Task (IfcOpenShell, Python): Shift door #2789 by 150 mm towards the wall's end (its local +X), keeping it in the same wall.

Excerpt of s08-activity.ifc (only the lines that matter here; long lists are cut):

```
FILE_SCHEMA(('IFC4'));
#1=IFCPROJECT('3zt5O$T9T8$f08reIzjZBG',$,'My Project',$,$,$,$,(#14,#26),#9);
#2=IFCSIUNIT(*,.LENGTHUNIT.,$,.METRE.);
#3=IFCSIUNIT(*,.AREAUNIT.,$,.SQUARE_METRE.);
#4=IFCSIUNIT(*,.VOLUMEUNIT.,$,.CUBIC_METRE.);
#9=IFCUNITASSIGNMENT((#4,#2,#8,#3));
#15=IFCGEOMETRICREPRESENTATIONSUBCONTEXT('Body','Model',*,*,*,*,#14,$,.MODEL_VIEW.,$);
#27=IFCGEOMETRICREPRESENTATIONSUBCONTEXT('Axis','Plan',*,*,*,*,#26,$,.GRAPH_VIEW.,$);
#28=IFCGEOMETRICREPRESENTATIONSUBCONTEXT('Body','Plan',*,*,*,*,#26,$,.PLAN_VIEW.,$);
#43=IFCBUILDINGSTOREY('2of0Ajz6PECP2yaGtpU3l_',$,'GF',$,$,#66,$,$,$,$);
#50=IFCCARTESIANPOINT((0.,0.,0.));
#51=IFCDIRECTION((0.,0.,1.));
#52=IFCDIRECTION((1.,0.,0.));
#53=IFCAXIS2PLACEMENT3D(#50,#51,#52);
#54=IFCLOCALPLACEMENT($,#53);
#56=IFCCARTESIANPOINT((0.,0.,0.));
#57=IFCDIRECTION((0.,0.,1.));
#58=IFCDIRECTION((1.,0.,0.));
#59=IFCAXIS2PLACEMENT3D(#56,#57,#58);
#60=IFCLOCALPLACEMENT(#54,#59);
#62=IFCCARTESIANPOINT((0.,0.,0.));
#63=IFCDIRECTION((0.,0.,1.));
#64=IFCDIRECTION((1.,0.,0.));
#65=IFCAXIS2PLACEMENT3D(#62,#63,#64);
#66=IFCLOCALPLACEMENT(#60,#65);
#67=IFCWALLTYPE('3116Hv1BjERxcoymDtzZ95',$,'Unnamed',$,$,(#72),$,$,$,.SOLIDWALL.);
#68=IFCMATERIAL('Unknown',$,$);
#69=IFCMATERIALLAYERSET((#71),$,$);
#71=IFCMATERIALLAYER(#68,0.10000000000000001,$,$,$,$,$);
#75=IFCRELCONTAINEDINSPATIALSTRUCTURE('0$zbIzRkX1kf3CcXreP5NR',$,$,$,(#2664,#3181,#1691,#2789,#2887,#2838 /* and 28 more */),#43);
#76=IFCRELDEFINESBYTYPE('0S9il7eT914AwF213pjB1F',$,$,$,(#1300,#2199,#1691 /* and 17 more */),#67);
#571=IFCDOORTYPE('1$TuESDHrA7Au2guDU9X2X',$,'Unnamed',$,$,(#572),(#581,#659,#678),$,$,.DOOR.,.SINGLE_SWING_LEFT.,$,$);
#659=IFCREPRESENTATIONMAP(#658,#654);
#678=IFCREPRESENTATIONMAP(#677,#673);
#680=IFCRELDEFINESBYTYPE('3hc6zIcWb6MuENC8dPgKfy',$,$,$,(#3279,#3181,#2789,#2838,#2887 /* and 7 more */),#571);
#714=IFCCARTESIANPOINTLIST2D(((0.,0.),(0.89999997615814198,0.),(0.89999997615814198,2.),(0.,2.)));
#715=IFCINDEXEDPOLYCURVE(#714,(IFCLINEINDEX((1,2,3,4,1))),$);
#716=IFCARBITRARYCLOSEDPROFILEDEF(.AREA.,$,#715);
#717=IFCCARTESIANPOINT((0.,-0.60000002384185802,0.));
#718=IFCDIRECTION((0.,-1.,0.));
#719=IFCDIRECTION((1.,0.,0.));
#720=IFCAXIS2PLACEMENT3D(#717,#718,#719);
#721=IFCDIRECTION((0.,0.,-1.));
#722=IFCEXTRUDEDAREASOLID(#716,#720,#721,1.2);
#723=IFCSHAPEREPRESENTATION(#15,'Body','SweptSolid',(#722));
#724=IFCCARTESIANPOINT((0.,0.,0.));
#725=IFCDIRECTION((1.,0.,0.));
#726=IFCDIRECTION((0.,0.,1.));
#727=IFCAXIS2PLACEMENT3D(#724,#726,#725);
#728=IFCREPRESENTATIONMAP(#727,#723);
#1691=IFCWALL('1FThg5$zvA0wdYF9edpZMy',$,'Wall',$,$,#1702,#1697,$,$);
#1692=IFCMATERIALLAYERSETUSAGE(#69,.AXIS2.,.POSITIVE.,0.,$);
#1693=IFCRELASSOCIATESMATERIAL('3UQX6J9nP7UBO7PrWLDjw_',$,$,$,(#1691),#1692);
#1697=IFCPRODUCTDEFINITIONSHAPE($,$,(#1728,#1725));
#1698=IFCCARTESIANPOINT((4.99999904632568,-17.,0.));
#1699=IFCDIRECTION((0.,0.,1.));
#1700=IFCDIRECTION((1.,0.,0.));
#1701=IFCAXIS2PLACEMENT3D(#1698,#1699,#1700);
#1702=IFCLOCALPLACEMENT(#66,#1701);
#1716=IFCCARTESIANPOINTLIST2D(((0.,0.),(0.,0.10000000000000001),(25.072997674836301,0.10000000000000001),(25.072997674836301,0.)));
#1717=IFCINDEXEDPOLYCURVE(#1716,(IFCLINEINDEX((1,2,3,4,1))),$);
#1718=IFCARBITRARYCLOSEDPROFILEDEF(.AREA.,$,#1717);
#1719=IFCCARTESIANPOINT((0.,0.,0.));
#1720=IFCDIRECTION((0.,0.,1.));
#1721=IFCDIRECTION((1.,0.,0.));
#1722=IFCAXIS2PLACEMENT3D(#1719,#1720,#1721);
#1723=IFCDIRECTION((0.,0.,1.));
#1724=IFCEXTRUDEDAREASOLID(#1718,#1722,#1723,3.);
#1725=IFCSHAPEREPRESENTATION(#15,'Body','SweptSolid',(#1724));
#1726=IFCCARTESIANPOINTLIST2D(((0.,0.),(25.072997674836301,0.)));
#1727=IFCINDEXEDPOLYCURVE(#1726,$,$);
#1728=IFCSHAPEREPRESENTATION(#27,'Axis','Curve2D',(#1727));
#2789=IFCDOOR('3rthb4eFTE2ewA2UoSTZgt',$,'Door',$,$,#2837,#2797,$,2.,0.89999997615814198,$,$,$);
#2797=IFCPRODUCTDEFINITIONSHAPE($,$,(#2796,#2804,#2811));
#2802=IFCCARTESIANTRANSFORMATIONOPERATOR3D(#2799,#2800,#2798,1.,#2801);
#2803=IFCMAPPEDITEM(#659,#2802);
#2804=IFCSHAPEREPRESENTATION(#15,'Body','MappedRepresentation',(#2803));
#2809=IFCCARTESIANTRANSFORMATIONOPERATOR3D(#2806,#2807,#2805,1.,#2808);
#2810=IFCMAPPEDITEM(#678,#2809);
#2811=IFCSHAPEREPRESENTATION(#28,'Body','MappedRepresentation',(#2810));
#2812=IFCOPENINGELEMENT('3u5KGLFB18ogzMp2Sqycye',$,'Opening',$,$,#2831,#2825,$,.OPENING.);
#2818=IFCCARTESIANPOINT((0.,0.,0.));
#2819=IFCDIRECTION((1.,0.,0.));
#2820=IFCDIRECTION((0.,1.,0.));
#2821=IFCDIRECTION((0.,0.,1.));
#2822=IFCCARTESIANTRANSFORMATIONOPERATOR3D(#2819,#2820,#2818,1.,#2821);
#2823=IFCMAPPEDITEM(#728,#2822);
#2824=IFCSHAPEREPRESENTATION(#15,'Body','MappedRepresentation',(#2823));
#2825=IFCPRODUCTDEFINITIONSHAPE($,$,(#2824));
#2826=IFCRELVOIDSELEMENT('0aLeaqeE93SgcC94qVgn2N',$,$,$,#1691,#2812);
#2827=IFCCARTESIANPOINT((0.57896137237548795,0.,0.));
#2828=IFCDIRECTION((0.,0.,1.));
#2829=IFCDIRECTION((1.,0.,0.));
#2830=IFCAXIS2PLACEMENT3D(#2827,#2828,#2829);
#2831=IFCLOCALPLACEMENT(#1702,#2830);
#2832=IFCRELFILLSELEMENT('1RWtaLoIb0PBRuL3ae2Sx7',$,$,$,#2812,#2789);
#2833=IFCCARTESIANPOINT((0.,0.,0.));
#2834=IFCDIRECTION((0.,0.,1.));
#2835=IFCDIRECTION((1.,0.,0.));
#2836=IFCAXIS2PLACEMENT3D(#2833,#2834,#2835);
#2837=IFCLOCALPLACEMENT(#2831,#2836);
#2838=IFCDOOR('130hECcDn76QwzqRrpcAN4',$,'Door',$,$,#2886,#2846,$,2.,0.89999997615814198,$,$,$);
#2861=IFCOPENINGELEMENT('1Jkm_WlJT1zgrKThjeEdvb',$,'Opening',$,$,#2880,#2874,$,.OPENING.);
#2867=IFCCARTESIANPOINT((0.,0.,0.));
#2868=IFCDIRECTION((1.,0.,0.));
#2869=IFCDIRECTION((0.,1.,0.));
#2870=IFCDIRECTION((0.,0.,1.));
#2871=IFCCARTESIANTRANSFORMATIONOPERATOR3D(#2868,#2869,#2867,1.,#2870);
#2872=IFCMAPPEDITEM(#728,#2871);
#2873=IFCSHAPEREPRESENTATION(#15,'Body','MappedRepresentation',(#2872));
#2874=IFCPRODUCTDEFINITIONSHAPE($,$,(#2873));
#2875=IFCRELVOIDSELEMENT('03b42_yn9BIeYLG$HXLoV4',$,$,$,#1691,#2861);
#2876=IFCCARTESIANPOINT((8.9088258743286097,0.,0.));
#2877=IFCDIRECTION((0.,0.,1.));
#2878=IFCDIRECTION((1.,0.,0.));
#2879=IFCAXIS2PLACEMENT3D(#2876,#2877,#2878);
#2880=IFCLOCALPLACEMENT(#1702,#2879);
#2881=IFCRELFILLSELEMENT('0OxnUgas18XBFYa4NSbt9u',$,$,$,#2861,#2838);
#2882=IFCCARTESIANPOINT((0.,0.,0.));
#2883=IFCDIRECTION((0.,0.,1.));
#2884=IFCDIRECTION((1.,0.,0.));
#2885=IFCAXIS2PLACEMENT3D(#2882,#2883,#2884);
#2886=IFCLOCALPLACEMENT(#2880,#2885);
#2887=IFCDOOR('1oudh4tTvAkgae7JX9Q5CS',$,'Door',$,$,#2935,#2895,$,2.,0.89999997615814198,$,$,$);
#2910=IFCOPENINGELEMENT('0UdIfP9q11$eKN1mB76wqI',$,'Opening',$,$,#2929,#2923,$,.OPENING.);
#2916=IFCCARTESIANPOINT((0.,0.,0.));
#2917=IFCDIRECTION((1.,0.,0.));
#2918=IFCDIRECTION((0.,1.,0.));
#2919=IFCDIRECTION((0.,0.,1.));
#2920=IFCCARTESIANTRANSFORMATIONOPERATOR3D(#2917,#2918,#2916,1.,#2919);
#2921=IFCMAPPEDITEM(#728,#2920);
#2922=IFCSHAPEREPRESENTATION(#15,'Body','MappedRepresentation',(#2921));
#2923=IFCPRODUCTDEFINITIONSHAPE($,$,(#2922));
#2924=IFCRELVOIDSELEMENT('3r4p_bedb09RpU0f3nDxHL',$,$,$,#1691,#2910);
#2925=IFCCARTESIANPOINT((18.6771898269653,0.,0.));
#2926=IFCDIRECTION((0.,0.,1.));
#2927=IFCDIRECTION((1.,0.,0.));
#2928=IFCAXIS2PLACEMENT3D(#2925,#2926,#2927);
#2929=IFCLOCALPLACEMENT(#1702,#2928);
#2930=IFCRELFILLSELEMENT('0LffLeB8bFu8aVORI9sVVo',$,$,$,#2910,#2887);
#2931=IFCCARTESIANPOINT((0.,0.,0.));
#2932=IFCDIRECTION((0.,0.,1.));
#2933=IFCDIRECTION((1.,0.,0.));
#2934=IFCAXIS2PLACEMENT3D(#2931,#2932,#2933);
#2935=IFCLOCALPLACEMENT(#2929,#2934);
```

```python
import ifcopenshell
import ifcopenshell.api.geometry
import ifcopenshell.util.placement

model = ifcopenshell.open("s08-activity.ifc")

door = model.by_guid("3rthb4eFTE2ewA2UoSTZgt")
opening = door.FillsVoids[0].RelatingOpeningElement
wall = opening.VoidsElements[0].RelatingBuildingElement

wall_matrix = ifcopenshell.util.placement.get_local_placement(wall.ObjectPlacement)
shift = wall_matrix[:3, 0] * 0.15
before = ifcopenshell.util.placement.get_local_placement(door.ObjectPlacement)[:3, 3].copy()

# The door is placed relative to its opening, so it follows when the opening moves.
matrix = ifcopenshell.util.placement.get_local_placement(opening.ObjectPlacement)
matrix[:3, 3] += shift
ifcopenshell.api.geometry.edit_object_placement(
    model, product=opening, matrix=matrix, is_si=False, should_transform_children=True
)

after = ifcopenshell.util.placement.get_local_placement(door.ObjectPlacement)[:3, 3]
print("door moved by", (after - before).round(3) + 0.0)

model.write("s08-activity_updated.ifc")
```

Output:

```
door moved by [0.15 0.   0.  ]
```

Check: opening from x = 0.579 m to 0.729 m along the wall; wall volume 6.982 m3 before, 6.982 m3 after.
